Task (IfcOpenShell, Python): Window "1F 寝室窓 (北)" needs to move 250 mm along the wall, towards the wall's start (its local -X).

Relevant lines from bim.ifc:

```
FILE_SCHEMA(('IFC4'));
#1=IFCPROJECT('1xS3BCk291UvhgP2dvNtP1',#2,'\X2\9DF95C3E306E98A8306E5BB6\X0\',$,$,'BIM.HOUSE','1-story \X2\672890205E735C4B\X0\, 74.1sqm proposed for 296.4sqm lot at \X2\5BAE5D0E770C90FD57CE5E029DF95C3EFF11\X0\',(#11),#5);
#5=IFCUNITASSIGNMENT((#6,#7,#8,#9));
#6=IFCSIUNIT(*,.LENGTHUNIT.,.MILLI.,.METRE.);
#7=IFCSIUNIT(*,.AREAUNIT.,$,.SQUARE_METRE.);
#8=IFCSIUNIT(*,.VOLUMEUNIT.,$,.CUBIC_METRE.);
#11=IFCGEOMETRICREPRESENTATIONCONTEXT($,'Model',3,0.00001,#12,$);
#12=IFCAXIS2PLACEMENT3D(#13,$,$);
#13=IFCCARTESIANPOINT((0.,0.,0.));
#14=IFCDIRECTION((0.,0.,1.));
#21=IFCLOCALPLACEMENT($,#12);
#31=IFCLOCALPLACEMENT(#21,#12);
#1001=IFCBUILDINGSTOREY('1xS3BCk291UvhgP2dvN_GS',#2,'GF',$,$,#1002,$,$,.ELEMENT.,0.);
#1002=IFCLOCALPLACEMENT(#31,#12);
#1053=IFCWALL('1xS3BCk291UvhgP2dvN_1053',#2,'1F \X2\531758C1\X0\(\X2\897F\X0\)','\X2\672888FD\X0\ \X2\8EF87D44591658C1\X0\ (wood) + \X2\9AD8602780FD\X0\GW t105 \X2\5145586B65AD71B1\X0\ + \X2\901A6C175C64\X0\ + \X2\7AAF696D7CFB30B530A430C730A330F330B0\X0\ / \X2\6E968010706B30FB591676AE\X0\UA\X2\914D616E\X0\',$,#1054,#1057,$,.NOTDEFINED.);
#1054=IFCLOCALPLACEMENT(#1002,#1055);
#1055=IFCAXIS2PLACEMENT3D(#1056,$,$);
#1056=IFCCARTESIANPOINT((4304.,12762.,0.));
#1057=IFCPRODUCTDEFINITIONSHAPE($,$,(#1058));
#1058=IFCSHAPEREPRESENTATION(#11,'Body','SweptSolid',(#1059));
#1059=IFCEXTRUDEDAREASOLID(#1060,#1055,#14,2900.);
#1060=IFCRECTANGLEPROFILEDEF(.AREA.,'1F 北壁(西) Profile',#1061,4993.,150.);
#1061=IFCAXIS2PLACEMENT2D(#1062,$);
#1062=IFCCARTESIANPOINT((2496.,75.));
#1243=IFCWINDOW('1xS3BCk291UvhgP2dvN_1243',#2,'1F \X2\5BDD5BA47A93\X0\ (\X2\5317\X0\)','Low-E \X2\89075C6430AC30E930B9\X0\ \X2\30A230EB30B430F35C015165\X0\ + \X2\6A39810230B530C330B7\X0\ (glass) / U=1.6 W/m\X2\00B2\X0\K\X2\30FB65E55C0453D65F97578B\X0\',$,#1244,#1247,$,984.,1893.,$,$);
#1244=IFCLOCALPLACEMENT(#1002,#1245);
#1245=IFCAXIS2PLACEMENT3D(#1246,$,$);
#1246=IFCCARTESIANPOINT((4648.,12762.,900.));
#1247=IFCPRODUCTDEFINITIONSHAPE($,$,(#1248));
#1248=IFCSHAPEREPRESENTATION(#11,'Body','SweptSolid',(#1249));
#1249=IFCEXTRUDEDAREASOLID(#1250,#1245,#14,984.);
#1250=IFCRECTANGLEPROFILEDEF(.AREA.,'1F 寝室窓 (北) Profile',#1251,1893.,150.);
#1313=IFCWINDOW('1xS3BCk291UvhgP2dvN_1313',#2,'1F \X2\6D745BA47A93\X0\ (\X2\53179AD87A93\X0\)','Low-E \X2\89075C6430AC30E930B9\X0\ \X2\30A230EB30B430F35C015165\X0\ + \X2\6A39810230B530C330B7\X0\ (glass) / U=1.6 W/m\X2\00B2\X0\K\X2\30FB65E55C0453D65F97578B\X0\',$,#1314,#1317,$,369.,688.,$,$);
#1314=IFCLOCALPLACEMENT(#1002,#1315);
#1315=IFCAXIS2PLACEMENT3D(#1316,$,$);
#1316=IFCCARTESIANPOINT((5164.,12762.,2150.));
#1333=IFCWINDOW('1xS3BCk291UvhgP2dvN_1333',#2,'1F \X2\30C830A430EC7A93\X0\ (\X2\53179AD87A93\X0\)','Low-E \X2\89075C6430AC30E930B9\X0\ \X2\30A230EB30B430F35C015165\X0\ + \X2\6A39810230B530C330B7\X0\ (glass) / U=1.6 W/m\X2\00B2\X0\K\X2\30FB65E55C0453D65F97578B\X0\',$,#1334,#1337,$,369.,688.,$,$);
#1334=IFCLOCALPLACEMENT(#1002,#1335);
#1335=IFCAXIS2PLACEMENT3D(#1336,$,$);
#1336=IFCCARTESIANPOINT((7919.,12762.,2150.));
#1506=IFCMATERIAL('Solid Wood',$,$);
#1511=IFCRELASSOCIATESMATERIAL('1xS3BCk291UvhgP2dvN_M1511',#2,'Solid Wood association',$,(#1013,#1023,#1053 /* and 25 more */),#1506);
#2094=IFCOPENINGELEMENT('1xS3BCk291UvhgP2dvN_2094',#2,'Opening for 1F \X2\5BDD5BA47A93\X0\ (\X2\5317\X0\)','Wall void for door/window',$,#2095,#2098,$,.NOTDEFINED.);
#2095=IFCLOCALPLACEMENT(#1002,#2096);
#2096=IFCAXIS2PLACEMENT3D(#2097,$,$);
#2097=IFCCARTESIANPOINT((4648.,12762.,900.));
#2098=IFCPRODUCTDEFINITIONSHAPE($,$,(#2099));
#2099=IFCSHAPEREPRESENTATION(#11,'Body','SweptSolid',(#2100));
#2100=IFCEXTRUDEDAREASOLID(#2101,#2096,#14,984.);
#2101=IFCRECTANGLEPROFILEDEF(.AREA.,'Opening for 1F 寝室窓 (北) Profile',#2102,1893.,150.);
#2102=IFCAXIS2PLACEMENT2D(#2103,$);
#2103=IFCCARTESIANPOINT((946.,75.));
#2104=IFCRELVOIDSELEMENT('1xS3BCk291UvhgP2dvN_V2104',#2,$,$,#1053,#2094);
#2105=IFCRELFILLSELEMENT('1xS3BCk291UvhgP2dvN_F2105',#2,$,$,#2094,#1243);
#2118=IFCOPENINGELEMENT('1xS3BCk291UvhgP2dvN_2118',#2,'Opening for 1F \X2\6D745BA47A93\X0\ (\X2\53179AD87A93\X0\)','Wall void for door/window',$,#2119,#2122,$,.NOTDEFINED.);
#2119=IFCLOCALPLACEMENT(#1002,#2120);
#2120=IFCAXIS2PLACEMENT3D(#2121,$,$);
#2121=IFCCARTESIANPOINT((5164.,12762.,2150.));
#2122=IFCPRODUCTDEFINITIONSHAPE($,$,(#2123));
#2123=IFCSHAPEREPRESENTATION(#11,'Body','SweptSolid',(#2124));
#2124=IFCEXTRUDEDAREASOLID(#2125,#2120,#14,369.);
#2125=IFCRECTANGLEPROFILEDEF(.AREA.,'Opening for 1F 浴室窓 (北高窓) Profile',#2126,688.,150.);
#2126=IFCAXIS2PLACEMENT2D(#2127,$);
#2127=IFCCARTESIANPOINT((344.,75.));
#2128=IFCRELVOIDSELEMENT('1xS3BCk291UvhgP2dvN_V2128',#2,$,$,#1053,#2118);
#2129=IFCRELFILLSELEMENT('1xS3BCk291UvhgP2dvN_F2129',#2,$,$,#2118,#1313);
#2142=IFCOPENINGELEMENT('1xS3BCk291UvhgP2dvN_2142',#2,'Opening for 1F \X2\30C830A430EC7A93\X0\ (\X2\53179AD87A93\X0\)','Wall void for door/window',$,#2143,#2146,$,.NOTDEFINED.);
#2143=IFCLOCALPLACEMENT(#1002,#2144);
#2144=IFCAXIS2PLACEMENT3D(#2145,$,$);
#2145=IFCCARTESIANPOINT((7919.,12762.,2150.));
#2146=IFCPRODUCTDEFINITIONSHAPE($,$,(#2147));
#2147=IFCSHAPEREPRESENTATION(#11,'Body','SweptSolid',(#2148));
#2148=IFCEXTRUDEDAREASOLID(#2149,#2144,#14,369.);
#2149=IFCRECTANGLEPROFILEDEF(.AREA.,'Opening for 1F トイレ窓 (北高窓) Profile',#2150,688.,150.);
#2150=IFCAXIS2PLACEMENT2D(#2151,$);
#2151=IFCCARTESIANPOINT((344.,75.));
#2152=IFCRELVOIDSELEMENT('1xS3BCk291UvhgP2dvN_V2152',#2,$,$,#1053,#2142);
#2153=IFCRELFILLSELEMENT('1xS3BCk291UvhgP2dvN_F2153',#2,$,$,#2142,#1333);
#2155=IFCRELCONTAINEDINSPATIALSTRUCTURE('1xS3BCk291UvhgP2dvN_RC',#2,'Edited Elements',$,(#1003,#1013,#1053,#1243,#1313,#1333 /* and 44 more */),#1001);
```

```python
import ifcopenshell
import ifcopenshell.api.geometry
import ifcopenshell.util.placement
import ifcopenshell.util.unit

model = ifcopenshell.open("bim.ifc")
unit_scale = ifcopenshell.util.unit.calculate_unit_scale(model)

window = model.by_guid("1xS3BCk291UvhgP2dvN_1243")
opening = window.FillsVoids[0].RelatingOpeningElement
wall = opening.VoidsElements[0].RelatingBuildingElement

wall_matrix = ifcopenshell.util.placement.get_local_placement(wall.ObjectPlacement)
shift = wall_matrix[:3, 0] * -0.25 / unit_scale
before = ifcopenshell.util.placement.get_local_placement(window.ObjectPlacement)[:3, 3].copy()

# The window is not placed relative to its opening, so move both.
for product in (opening, window):
    matrix = ifcopenshell.util.placement.get_local_placement(product.ObjectPlacement)
    matrix[:3, 3] += shift
    ifcopenshell.api.geometry.edit_object_placement(model, product=product, matrix=matrix, is_si=False)

after = ifcopenshell.util.placement.get_local_placement(window.ObjectPlacement)[:3, 3]
print("window moved by", (after - before).round(3) + 0.0)

model.write("bim_edited.ifc")
```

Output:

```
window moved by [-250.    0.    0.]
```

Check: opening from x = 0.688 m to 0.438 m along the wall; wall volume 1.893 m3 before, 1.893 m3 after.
